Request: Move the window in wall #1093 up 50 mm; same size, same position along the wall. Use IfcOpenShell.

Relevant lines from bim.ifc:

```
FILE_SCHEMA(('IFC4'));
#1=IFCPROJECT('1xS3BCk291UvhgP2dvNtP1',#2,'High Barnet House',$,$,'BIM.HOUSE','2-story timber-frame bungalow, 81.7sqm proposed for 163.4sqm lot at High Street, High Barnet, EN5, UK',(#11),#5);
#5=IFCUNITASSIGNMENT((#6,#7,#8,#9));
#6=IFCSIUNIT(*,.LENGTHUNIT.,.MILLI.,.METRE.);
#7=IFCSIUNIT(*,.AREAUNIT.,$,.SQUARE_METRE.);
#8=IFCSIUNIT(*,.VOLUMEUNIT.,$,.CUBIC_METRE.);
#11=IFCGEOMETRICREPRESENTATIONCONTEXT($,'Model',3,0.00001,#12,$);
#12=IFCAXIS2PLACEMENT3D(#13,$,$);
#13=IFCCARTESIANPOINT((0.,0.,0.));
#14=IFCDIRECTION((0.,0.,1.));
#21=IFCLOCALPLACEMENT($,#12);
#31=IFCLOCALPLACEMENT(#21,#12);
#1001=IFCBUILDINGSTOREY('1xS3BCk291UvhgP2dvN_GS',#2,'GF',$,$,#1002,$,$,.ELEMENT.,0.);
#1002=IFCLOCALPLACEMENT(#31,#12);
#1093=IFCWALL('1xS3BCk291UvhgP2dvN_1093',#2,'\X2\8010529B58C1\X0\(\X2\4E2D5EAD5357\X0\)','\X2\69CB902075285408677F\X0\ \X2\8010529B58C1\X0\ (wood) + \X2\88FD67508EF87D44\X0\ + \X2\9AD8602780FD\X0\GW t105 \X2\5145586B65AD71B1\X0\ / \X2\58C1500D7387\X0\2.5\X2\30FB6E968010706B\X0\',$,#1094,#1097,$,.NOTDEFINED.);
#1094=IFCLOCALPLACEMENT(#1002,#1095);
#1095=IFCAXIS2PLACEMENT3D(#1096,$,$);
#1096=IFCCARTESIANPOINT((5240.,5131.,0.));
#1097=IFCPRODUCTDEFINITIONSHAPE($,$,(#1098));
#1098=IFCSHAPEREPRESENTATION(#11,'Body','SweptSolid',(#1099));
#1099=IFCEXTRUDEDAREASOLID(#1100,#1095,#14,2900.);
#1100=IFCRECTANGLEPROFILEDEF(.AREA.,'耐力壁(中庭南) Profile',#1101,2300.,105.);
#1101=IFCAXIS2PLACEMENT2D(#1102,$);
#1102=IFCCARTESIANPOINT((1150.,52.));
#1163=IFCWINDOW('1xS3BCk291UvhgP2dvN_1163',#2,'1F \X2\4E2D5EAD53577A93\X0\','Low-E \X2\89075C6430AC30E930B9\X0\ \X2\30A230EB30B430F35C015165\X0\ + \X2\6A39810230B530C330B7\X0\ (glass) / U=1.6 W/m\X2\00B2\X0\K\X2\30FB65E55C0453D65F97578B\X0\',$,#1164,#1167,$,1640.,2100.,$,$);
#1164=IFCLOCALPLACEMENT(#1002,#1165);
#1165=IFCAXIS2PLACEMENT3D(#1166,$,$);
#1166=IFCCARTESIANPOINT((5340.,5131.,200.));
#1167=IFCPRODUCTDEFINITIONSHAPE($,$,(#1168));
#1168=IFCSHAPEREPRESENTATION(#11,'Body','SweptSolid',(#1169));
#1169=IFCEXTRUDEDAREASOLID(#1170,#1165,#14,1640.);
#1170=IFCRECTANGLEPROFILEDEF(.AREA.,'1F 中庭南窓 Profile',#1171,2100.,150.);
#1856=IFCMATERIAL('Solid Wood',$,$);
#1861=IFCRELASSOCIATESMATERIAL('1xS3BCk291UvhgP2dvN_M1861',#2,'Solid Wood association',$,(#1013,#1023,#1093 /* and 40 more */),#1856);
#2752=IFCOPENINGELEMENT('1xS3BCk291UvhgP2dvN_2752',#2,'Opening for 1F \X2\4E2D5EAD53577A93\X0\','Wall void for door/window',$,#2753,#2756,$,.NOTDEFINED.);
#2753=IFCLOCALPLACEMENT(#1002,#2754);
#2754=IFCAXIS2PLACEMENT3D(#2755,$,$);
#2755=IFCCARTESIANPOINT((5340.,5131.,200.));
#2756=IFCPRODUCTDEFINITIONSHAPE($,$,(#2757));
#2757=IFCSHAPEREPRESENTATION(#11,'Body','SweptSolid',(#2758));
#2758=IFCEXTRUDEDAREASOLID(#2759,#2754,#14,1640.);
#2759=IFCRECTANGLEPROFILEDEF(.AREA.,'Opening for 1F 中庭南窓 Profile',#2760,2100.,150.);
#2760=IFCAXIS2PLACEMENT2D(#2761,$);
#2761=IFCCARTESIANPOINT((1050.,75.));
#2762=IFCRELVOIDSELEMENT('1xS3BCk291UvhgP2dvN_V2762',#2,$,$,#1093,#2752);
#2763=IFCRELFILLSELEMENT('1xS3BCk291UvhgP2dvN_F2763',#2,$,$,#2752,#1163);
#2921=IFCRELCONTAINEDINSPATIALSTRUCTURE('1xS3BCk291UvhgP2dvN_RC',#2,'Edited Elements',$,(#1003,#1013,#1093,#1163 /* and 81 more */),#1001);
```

```python
import numpy as np
import ifcopenshell
import ifcopenshell.api.geometry
import ifcopenshell.util.placement
import ifcopenshell.util.unit

model = ifcopenshell.open("bim.ifc")
unit_scale = ifcopenshell.util.unit.calculate_unit_scale(model)

window = model.by_id(1163)
opening = window.FillsVoids[0].RelatingOpeningElement
dz = 0.05 / unit_scale

shift = np.array([0.0, 0.0, dz])
# The window is not placed relative to its opening, so move both.
for product in (opening, window):
    matrix = ifcopenshell.util.placement.get_local_placement(product.ObjectPlacement)
    matrix[:3, 3] += shift
    ifcopenshell.api.geometry.edit_object_placement(model, product=product, matrix=matrix, is_si=False)

print(f"moved by {dz * unit_scale:+.3f} m")

model.write("bim_v2.ifc")
```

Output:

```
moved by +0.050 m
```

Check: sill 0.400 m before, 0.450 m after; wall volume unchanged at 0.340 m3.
